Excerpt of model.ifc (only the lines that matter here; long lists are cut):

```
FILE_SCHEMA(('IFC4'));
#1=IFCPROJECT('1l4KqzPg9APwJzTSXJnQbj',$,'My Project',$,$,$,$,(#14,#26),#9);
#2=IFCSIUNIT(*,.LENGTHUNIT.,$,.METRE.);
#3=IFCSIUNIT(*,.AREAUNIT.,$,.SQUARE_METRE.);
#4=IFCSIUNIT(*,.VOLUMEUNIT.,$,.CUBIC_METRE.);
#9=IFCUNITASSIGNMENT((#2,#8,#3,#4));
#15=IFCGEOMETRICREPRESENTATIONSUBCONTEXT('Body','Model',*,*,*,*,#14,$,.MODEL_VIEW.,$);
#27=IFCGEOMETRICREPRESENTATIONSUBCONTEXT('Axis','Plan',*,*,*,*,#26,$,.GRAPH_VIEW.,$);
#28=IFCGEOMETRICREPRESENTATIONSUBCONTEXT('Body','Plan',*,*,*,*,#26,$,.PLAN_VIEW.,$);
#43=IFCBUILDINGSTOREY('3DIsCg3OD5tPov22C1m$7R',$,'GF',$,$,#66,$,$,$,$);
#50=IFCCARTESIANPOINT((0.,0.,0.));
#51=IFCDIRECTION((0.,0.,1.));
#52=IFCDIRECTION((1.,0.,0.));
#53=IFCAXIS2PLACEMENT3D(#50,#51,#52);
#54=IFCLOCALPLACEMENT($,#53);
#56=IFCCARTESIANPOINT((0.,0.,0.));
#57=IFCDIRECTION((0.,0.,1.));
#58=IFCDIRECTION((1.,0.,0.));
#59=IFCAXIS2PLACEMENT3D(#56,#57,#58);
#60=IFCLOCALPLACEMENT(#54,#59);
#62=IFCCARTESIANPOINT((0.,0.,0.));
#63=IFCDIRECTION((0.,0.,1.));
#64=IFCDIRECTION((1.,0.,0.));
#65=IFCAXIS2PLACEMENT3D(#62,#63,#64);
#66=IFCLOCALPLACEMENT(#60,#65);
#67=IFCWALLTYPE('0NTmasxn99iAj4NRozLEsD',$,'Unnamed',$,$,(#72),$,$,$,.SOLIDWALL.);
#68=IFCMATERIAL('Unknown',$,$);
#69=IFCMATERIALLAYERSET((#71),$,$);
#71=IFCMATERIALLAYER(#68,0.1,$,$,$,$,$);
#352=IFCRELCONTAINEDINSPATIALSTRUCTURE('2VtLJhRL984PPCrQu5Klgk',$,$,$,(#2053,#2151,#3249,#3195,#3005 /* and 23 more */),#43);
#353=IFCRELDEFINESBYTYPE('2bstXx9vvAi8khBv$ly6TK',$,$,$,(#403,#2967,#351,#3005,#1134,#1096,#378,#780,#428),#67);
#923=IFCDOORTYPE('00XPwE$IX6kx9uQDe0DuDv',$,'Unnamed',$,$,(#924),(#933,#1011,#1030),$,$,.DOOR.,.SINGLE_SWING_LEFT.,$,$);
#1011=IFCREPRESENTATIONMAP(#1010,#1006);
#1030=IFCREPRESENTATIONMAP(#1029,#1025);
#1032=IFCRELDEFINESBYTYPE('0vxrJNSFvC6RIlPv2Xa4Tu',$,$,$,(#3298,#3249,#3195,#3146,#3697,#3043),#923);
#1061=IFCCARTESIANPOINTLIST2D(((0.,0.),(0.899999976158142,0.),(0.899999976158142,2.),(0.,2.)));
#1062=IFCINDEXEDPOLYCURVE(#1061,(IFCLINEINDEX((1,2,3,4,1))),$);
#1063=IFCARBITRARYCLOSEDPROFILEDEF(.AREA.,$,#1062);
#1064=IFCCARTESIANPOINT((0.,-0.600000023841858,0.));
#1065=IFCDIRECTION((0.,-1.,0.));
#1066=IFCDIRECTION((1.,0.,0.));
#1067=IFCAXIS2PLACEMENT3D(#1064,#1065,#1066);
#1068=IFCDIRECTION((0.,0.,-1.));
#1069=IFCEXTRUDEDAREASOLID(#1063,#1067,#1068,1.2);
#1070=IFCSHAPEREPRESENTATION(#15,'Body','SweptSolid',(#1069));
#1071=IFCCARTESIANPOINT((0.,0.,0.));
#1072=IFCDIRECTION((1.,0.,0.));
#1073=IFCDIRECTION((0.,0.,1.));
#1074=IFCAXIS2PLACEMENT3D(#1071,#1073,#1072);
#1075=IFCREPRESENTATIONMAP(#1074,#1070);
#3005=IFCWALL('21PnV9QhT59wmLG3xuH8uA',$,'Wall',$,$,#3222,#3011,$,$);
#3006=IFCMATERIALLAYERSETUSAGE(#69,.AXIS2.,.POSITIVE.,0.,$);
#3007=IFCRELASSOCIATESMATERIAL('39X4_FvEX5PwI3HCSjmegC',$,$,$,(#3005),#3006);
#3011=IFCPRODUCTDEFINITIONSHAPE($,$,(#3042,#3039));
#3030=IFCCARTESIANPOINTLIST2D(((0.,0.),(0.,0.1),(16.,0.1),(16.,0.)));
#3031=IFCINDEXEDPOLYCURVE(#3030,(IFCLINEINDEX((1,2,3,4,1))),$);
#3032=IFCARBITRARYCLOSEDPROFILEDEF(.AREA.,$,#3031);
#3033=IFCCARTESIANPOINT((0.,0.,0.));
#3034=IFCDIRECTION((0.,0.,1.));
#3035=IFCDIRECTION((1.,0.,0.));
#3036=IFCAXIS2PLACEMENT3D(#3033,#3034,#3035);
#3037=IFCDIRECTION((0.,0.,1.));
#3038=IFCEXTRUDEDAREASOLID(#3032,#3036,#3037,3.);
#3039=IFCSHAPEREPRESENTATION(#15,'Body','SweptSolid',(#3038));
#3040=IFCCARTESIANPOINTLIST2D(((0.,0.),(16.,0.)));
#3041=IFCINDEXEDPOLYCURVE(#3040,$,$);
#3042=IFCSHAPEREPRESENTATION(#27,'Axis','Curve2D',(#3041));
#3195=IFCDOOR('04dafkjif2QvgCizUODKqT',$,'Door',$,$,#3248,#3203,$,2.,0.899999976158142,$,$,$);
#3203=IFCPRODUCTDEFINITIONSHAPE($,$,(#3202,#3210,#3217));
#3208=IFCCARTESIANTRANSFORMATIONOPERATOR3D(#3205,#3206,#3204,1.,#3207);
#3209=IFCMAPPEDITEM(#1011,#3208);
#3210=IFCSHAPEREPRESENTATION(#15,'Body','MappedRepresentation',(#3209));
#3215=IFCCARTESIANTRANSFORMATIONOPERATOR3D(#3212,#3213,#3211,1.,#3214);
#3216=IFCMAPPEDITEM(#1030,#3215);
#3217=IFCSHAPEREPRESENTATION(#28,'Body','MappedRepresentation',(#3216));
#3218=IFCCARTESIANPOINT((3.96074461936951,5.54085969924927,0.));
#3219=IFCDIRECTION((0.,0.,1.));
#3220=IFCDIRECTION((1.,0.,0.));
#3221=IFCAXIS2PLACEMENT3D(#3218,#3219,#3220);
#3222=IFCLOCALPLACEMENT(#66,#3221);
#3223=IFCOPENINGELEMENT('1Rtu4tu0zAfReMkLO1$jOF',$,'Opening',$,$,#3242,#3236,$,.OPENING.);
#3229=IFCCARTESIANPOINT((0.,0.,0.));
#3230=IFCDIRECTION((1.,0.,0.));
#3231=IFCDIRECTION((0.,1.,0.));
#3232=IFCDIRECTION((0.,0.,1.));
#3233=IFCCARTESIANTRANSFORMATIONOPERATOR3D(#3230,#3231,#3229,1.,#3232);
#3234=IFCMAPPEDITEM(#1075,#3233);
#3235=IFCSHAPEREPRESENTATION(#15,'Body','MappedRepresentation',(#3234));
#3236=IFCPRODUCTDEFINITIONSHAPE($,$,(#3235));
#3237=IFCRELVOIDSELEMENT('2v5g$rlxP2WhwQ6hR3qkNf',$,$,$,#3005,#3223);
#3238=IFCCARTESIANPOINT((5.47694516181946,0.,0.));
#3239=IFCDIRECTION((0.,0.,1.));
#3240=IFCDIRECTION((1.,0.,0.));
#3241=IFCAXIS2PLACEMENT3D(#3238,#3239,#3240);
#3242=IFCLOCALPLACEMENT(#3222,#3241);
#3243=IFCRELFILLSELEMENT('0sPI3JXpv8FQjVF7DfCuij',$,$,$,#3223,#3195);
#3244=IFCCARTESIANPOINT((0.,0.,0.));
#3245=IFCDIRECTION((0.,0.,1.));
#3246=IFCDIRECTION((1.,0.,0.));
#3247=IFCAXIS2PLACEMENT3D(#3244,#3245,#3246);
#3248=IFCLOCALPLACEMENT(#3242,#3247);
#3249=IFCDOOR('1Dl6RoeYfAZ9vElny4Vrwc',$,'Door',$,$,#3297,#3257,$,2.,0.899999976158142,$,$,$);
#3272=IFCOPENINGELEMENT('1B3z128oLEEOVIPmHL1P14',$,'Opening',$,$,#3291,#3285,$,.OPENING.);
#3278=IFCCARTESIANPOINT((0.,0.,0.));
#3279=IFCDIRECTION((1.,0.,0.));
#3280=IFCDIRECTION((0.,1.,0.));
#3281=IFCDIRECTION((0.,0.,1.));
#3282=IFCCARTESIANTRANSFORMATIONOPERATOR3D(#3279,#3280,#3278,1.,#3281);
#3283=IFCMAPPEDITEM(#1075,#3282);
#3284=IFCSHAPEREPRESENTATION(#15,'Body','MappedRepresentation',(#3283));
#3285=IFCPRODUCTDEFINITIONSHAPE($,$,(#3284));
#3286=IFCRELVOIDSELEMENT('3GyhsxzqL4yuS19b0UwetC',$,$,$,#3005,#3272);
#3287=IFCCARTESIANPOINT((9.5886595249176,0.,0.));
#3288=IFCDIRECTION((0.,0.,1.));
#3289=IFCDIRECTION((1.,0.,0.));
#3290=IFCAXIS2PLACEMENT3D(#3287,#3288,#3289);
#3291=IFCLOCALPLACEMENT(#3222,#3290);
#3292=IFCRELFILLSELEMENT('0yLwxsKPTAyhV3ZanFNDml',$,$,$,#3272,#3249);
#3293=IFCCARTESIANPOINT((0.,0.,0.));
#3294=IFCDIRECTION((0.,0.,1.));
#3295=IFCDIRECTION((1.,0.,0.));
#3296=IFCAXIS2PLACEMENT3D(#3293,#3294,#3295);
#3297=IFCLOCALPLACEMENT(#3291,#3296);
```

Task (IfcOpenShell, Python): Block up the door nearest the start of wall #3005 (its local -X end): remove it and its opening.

```python
import ifcopenshell
import ifcopenshell.api.feature
import ifcopenshell.api.root
import ifcopenshell.geom
import ifcopenshell.util.shape

model = ifcopenshell.open("model.ifc")
settings = ifcopenshell.geom.settings()


def volume(element):
    """Net volume in cubic metres, openings subtracted."""
    shape = ifcopenshell.geom.create_shape(settings, element)
    return ifcopenshell.util.shape.get_volume(shape.geometry)


door = model.by_guid("04dafkjif2QvgCizUODKqT")
opening = door.FillsVoids[0].RelatingOpeningElement
wall = opening.VoidsElements[0].RelatingBuildingElement
before = volume(wall)

ifcopenshell.api.root.remove_product(model, product=door)
ifcopenshell.api.feature.remove_feature(model, feature=opening)

after = volume(wall)

print(f"wall volume {before:.3f} -> {after:.3f} m3")

model.write("model_rev.ifc")
```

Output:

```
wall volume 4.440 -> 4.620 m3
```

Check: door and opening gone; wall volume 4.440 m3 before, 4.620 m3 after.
